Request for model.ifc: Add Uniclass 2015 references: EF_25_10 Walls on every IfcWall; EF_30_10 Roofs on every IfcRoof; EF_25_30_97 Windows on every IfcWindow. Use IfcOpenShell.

First a look at what the model holds.

```python
import ifcopenshell

model = ifcopenshell.open("model.ifc")
print(model.schema)
print("classifications:", [c.Name for c in model.by_type("IfcClassification")])
for ifc_class in ("IfcDoor", "IfcRoof", "IfcStair", "IfcWall", "IfcWindow"):
    print(ifc_class, len(model.by_type(ifc_class)))
```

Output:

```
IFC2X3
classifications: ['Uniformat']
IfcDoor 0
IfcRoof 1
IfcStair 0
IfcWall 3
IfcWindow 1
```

```python
import ifcopenshell
import ifcopenshell.api.classification

model = ifcopenshell.open("model.ifc")

# IFC2X3 requires Source and Edition and has no link from the project to the system.
system = model.create_entity("IfcClassification", Source="NBS", Edition="2015", Name="Uniclass 2015")

codes = {
    "IfcWall": ("EF_25_10", "Walls"),
    "IfcRoof": ("EF_30_10", "Roofs"),
    "IfcWindow": ("EF_25_30_97", "Windows"),
}
for ifc_class, (code, name) in codes.items():
    products = model.by_type(ifc_class)
    ifcopenshell.api.classification.add_reference(
        model, products=products, classification=system, identification=code, name=name
    )
    print(code, len(products))

model.write("model_v2.ifc")
```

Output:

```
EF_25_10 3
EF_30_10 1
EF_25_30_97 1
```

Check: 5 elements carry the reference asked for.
